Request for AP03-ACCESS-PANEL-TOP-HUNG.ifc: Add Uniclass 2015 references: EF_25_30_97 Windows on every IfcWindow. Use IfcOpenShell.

First a look at what the model holds.

```python
import ifcopenshell

model = ifcopenshell.open("AP03-ACCESS-PANEL-TOP-HUNG.ifc")
print(model.schema)
print("classifications:", [c.Name for c in model.by_type("IfcClassification")])
for ifc_class in ("IfcDoor", "IfcRoof", "IfcStair", "IfcWall", "IfcWindow"):
    print(ifc_class, len(model.by_type(ifc_class)))
```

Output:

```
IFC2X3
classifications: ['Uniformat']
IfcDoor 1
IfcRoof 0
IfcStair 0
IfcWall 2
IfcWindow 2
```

```python
import ifcopenshell
import ifcopenshell.api.classification

model = ifcopenshell.open("AP03-ACCESS-PANEL-TOP-HUNG.ifc")

# IFC2X3 requires Source and Edition and has no link from the project to the system.
system = model.create_entity("IfcClassification", Source="NBS", Edition="2015", Name="Uniclass 2015")

codes = {
    "IfcWindow": ("EF_25_30_97", "Windows"),
}
for ifc_class, (code, name) in codes.items():
    products = model.by_type(ifc_class)
    ifcopenshell.api.classification.add_reference(
        model, products=products, classification=system, identification=code, name=name
    )
    print(code, len(products))

model.write("AP03-ACCESS-PANEL-TOP-HUNG_rev.ifc")
```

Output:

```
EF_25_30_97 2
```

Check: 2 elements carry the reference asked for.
